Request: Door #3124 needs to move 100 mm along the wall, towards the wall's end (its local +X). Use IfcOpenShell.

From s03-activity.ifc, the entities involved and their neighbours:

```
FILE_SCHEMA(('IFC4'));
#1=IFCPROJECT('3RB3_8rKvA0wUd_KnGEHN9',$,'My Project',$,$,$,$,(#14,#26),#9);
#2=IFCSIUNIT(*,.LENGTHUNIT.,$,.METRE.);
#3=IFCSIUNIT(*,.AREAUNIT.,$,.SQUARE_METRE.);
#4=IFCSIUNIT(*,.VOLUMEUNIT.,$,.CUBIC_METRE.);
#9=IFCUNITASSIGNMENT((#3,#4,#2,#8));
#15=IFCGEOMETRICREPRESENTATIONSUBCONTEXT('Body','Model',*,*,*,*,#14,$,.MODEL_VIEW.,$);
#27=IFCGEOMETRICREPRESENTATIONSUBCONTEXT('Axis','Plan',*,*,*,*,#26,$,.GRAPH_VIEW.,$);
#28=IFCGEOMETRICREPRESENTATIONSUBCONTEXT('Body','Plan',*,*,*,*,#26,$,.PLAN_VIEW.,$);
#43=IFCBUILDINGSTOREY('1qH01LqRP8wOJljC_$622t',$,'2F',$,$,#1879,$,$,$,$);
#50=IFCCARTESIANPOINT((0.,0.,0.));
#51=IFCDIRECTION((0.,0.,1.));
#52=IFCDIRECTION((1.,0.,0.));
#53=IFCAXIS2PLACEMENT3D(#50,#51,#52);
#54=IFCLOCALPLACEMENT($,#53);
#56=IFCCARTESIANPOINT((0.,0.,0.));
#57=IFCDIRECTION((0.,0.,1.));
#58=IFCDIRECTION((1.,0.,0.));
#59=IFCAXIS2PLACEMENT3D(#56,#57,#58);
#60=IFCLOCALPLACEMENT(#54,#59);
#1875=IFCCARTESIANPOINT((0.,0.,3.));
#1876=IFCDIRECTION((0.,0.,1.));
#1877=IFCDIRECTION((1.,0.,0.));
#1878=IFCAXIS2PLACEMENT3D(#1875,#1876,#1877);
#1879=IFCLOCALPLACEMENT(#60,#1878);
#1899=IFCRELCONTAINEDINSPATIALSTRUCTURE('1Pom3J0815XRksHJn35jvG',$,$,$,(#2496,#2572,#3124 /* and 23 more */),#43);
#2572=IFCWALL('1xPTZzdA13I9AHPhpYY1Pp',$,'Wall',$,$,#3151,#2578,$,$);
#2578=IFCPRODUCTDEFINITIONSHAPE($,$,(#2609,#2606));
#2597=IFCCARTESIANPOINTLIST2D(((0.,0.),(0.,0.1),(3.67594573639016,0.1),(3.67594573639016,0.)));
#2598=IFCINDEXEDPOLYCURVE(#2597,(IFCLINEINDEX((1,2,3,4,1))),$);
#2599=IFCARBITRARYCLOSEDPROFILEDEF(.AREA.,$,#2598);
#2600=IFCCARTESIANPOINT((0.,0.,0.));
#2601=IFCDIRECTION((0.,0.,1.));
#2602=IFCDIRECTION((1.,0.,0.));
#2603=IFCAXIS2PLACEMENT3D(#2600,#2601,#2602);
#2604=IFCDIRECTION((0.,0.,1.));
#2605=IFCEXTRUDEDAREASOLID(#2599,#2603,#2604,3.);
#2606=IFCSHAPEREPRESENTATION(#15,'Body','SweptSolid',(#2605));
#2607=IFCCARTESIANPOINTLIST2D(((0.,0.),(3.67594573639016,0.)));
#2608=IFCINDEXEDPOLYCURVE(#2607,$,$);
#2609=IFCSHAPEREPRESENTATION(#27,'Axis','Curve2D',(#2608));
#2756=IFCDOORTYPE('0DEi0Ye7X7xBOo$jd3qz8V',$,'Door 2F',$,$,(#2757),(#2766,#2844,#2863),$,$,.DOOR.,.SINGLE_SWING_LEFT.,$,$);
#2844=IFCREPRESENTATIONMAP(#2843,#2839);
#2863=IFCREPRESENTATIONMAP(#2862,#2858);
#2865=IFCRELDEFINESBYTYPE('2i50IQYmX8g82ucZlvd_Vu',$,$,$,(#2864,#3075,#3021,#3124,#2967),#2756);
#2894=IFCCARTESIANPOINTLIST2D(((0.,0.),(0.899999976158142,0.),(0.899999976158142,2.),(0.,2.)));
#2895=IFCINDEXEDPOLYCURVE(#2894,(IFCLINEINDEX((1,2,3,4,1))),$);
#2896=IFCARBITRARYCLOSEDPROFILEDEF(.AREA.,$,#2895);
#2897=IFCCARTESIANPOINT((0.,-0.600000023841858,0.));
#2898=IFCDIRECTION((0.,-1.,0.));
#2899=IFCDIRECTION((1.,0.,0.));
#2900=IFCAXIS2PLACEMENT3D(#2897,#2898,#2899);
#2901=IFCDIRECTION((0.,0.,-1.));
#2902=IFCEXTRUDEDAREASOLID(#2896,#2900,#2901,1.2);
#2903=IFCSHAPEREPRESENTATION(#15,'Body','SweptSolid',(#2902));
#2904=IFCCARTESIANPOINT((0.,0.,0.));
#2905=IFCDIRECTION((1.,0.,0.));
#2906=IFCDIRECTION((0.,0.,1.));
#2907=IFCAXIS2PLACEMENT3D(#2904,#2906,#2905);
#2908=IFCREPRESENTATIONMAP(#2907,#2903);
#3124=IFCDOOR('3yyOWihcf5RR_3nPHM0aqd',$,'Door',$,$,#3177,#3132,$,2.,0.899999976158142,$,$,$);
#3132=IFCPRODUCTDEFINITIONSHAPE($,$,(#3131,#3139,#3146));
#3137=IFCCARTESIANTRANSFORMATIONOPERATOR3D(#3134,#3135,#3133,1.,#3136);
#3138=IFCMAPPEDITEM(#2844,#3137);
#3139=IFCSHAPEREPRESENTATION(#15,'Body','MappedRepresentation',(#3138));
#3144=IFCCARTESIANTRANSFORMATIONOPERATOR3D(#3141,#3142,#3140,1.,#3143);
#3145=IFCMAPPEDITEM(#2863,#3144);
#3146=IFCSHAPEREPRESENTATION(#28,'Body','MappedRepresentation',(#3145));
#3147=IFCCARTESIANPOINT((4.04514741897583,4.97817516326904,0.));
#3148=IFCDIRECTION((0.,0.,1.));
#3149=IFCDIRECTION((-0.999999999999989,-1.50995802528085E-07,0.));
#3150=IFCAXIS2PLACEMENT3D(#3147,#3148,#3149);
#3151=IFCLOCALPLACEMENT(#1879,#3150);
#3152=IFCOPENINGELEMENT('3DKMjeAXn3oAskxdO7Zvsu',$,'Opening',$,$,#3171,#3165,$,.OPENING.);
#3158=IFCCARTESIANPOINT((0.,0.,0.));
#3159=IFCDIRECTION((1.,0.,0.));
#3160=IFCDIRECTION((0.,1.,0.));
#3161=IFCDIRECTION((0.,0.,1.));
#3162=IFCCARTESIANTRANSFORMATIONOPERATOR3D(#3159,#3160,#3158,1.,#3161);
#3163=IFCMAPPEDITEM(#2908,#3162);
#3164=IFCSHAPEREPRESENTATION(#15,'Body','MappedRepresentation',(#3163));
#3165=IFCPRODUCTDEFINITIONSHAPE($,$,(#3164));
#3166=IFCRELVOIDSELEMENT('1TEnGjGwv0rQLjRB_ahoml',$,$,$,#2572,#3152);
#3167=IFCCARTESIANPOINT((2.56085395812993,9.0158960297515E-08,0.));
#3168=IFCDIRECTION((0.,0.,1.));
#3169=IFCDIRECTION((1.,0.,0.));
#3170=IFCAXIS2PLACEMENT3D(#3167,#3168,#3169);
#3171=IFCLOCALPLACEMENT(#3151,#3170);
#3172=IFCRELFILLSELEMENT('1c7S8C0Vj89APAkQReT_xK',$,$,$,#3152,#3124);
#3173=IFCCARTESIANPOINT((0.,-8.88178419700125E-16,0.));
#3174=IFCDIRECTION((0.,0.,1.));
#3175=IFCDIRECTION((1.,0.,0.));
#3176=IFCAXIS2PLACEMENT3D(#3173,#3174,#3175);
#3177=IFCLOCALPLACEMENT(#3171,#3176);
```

```python
import ifcopenshell
import ifcopenshell.api.geometry
import ifcopenshell.util.placement
import ifcopenshell.util.unit

model = ifcopenshell.open("s03-activity.ifc")
unit_scale = ifcopenshell.util.unit.calculate_unit_scale(model)

door = model.by_guid("3yyOWihcf5RR_3nPHM0aqd")
opening = door.FillsVoids[0].RelatingOpeningElement
wall = opening.VoidsElements[0].RelatingBuildingElement

wall_matrix = ifcopenshell.util.placement.get_local_placement(wall.ObjectPlacement)
shift = wall_matrix[:3, 0] * 0.1 / unit_scale
before = ifcopenshell.util.placement.get_local_placement(door.ObjectPlacement)[:3, 3].copy()

# The door is placed relative to its opening, so it follows when the opening moves.
matrix = ifcopenshell.util.placement.get_local_placement(opening.ObjectPlacement)
matrix[:3, 3] += shift
ifcopenshell.api.geometry.edit_object_placement(
    model, product=opening, matrix=matrix, is_si=False, should_transform_children=True
)

after = ifcopenshell.util.placement.get_local_placement(door.ObjectPlacement)[:3, 3]
print("door moved by", (after - before).round(3) + 0.0)

model.write("s03-activity-out.ifc")
```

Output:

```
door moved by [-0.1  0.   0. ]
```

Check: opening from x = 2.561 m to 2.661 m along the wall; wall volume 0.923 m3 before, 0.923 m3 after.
